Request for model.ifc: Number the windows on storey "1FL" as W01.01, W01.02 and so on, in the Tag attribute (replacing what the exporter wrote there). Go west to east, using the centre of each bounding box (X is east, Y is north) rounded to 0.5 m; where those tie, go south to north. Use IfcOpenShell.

First a look at what the model holds.

```python
import ifcopenshell
import ifcopenshell.util.element
import ifcopenshell.util.placement

model = ifcopenshell.open("model.ifc")
print(model.schema)
storey = next(s for s in model.by_type("IfcBuildingStorey") if s.Name == "1FL")
windows = [e for e in ifcopenshell.util.element.get_decomposition(storey) if e.is_a("IfcWindow")]
for e in sorted(windows, key=lambda e: e.id()):
    origin = ifcopenshell.util.placement.get_local_placement(e.ObjectPlacement)[:3, 3]
    print(e.id(), e.Tag, e.Name, origin.round(2) + 0.0, sep=" | ")
```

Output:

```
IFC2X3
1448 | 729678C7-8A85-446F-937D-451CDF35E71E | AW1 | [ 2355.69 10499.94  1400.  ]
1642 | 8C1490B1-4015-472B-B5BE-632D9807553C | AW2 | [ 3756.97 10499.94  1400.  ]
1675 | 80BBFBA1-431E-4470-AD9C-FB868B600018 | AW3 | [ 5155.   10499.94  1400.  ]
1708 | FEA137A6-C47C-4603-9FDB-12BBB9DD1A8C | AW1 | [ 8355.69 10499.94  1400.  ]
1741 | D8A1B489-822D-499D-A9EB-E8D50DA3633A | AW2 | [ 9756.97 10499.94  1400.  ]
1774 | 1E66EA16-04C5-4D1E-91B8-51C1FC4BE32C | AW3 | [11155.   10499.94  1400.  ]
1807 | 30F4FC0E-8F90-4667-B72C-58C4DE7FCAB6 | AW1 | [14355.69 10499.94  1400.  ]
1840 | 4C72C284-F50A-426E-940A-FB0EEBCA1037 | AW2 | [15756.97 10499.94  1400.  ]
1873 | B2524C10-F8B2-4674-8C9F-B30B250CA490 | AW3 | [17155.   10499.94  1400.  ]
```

```python
import ifcopenshell
import ifcopenshell.geom
import ifcopenshell.util.element
import ifcopenshell.util.shape

model = ifcopenshell.open("model.ifc")
settings = ifcopenshell.geom.settings()
settings.set("use-world-coords", True)


def centre(element):
    shape = ifcopenshell.geom.create_shape(settings, element)
    return ifcopenshell.util.shape.get_bbox_centroid(shape.geometry)


storey = next(s for s in model.by_type("IfcBuildingStorey") if s.Name == "1FL")
windows = [e for e in ifcopenshell.util.element.get_decomposition(storey) if e.is_a("IfcWindow")]

# Insertion points can sit at a corner or the storey origin, so sort by the geometry (in metres).
centres = {e: centre(e) for e in windows}
windows.sort(key=lambda e: (round(centres[e][0] / 0.5), centres[e][1]))

for i, e in enumerate(windows, start=1):
    number = f"W01.{i:02d}"
    e.Tag = number
    print(e.id(), number)

model.write("model_rev.ifc")
```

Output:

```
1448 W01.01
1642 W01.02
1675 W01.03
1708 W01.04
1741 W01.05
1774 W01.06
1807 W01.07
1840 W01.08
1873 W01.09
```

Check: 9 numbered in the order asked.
